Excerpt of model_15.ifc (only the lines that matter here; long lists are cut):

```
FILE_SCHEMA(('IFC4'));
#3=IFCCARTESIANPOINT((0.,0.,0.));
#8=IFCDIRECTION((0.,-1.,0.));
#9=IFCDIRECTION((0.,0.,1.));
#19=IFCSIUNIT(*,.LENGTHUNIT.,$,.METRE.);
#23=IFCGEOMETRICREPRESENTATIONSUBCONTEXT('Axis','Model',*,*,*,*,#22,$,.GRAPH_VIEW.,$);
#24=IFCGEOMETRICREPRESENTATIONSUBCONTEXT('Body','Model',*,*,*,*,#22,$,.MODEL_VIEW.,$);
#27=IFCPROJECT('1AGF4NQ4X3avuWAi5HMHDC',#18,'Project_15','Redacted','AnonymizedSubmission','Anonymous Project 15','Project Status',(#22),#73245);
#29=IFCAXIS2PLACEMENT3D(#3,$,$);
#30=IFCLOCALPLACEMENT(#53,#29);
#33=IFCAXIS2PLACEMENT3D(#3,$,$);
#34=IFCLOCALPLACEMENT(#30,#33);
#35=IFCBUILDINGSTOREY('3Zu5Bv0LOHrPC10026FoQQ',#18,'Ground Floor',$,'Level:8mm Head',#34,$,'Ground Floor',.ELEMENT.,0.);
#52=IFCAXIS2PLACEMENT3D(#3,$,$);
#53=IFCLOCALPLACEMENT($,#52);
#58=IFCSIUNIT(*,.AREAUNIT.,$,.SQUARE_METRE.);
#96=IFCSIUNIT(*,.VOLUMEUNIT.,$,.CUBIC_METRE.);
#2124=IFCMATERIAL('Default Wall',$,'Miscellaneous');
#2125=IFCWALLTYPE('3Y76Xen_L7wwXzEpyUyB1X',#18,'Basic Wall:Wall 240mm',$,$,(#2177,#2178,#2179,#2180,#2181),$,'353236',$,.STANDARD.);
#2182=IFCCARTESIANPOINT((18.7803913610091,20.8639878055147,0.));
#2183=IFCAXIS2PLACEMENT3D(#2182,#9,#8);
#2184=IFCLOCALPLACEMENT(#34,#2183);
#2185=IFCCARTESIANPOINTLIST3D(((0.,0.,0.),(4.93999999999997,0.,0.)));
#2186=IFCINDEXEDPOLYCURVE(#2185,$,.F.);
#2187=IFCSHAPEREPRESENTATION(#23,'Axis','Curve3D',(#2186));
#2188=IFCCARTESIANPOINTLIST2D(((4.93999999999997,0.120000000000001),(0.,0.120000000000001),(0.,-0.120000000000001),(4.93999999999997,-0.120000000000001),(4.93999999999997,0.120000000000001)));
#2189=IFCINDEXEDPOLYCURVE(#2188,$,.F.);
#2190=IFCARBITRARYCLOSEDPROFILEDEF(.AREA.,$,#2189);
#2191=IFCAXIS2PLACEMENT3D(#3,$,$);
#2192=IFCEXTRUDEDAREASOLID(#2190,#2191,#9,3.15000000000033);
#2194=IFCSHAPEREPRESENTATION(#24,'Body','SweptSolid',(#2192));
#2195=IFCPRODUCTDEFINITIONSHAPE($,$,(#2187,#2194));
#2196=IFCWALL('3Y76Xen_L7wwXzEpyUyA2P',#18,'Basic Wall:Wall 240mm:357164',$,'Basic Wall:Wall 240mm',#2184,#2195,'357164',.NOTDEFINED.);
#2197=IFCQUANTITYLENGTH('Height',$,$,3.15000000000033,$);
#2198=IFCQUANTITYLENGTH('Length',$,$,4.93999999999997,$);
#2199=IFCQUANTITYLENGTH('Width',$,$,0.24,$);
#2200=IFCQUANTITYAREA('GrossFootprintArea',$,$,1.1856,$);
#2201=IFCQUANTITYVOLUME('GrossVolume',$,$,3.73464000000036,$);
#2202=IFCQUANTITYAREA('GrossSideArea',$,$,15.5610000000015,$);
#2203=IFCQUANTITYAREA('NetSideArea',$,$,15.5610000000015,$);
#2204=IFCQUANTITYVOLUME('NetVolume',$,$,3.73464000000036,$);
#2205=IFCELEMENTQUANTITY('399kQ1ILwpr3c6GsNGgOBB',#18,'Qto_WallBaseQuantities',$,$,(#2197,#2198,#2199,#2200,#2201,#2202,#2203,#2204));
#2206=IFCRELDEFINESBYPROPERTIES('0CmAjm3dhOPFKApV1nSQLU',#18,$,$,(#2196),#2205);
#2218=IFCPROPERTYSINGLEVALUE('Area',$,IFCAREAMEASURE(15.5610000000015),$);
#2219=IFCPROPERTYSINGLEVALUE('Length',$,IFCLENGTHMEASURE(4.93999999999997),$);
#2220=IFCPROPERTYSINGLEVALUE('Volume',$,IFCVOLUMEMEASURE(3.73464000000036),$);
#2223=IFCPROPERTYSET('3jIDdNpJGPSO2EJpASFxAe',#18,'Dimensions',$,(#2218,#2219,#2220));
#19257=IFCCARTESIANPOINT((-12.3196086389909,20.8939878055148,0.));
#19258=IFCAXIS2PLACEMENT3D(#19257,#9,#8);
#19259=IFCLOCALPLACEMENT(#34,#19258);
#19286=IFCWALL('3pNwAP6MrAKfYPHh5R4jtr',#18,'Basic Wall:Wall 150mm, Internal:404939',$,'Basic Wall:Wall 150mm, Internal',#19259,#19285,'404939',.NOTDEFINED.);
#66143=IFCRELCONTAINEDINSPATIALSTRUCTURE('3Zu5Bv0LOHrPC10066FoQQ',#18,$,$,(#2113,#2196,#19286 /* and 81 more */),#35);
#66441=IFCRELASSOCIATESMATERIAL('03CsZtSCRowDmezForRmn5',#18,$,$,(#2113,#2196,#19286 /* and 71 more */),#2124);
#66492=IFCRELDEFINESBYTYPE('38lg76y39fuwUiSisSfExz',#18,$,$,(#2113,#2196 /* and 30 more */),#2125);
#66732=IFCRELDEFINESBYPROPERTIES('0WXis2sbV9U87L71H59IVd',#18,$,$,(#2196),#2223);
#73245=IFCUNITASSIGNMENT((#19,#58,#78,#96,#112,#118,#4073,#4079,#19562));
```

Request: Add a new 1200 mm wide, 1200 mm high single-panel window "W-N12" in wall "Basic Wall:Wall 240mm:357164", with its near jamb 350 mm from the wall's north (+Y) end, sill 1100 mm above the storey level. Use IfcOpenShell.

```python
import numpy as np
import ifcopenshell
import ifcopenshell.api.feature
import ifcopenshell.api.geometry
import ifcopenshell.api.pset
import ifcopenshell.api.root
import ifcopenshell.api.spatial
import ifcopenshell.geom
import ifcopenshell.util.element
import ifcopenshell.util.placement
import ifcopenshell.util.representation
import ifcopenshell.util.shape
import ifcopenshell.util.unit

model = ifcopenshell.open("model_15.ifc")
unit_scale = ifcopenshell.util.unit.calculate_unit_scale(model)
area_scale = ifcopenshell.util.unit.calculate_unit_scale(model, "AREAUNIT")
volume_scale = ifcopenshell.util.unit.calculate_unit_scale(model, "VOLUMEUNIT")
settings = ifcopenshell.geom.settings()


def volume(element):
    """Net volume in cubic metres, openings subtracted."""
    shape = ifcopenshell.geom.create_shape(settings, element)
    return ifcopenshell.util.shape.get_volume(shape.geometry)


wall = model.by_id(2196)
storey = ifcopenshell.util.element.get_container(wall, ifc_class="IfcBuildingStorey")
context = ifcopenshell.util.representation.get_context(model, "Model", "Body", "MODEL_VIEW")
before = volume(wall)

width, height, from_end, sill = 1.2, 1.2, 0.35, 1.1  # metres

# The wall runs along its own X axis, and the end named is its -X end.
wall_shape = ifcopenshell.geom.create_shape(settings, wall)
x, y, z = ifcopenshell.util.shape.get_vertices(wall_shape.geometry).T
start = x.min() + from_end
face, thickness = float(y.min()), float(y.max() - y.min())
wall_matrix = ifcopenshell.util.placement.get_local_placement(wall.ObjectPlacement)
level = ifcopenshell.util.placement.get_local_placement(storey.ObjectPlacement)[2, 3]


def in_wall(x, y):
    """Placement at x, y metres in the wall's axes, at sill height."""
    matrix = wall_matrix.copy()
    matrix[:, 3] = wall_matrix @ np.array([x / unit_scale, y / unit_scale, 0.0, 1.0])
    matrix[2, 3] = level + sill / unit_scale
    return matrix


# Opening: a box that overshoots both wall faces by 50 mm.
opening = ifcopenshell.api.root.create_entity(model, ifc_class="IfcOpeningElement", predefined_type="OPENING")
box = ifcopenshell.api.geometry.add_wall_representation(
    model, context=context, length=width, height=height, thickness=thickness + 0.1
)
ifcopenshell.api.geometry.assign_representation(model, product=opening, representation=box)
ifcopenshell.api.geometry.edit_object_placement(model, product=opening, matrix=in_wall(start, face - 0.05), is_si=False)
ifcopenshell.api.feature.add_feature(model, feature=opening, element=wall)

window = ifcopenshell.api.root.create_entity(model, ifc_class="IfcWindow", name="W-N12", predefined_type="WINDOW")
window.OverallWidth, window.OverallHeight = width / unit_scale, height / unit_scale
window.PartitioningType = "SINGLE_PANEL"
body = ifcopenshell.api.geometry.add_window_representation(
    model,
    context=context,
    overall_width=window.OverallWidth,
    overall_height=window.OverallHeight,
    partition_type="SINGLE_PANEL",
)
ifcopenshell.api.geometry.assign_representation(model, product=window, representation=body)
ifcopenshell.api.spatial.assign_container(model, products=[window], relating_structure=storey)
ifcopenshell.api.feature.add_filling(model, opening=opening, element=window)

# Centre the window in the wall's thickness.
ifcopenshell.api.geometry.edit_object_placement(model, product=window, matrix=in_wall(start, face), is_si=False)
window_shape = ifcopenshell.geom.create_shape(settings, window)
depth = ifcopenshell.util.shape.get_vertices(window_shape.geometry)[:, 1]
offset = face + thickness / 2 - (depth.min() + depth.max()) / 2
ifcopenshell.api.geometry.edit_object_placement(model, product=window, matrix=in_wall(start, offset), is_si=False)

after = volume(wall)

# Update the wall's stored quantities.
qto = model.by_id(ifcopenshell.util.element.get_pset(wall, "Qto_WallBaseQuantities", should_inherit=False)["id"])
ifcopenshell.api.pset.edit_qto(model, qto=qto, properties={
    "NetSideArea": after / thickness / area_scale,
    "NetVolume": after / volume_scale,
})
pset = model.by_id(ifcopenshell.util.element.get_pset(wall, "Dimensions", should_inherit=False)["id"])
ifcopenshell.api.pset.edit_pset(model, pset=pset, properties={
    "Area": model.create_entity("IfcAreaMeasure", after / thickness / area_scale),
    "Volume": model.create_entity("IfcVolumeMeasure", after / volume_scale),
})

print(f"wall volume {before:.3f} -> {after:.3f} m3")

model.write("model_15_updated.ifc")
```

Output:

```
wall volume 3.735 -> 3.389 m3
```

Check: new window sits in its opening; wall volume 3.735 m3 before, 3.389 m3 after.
